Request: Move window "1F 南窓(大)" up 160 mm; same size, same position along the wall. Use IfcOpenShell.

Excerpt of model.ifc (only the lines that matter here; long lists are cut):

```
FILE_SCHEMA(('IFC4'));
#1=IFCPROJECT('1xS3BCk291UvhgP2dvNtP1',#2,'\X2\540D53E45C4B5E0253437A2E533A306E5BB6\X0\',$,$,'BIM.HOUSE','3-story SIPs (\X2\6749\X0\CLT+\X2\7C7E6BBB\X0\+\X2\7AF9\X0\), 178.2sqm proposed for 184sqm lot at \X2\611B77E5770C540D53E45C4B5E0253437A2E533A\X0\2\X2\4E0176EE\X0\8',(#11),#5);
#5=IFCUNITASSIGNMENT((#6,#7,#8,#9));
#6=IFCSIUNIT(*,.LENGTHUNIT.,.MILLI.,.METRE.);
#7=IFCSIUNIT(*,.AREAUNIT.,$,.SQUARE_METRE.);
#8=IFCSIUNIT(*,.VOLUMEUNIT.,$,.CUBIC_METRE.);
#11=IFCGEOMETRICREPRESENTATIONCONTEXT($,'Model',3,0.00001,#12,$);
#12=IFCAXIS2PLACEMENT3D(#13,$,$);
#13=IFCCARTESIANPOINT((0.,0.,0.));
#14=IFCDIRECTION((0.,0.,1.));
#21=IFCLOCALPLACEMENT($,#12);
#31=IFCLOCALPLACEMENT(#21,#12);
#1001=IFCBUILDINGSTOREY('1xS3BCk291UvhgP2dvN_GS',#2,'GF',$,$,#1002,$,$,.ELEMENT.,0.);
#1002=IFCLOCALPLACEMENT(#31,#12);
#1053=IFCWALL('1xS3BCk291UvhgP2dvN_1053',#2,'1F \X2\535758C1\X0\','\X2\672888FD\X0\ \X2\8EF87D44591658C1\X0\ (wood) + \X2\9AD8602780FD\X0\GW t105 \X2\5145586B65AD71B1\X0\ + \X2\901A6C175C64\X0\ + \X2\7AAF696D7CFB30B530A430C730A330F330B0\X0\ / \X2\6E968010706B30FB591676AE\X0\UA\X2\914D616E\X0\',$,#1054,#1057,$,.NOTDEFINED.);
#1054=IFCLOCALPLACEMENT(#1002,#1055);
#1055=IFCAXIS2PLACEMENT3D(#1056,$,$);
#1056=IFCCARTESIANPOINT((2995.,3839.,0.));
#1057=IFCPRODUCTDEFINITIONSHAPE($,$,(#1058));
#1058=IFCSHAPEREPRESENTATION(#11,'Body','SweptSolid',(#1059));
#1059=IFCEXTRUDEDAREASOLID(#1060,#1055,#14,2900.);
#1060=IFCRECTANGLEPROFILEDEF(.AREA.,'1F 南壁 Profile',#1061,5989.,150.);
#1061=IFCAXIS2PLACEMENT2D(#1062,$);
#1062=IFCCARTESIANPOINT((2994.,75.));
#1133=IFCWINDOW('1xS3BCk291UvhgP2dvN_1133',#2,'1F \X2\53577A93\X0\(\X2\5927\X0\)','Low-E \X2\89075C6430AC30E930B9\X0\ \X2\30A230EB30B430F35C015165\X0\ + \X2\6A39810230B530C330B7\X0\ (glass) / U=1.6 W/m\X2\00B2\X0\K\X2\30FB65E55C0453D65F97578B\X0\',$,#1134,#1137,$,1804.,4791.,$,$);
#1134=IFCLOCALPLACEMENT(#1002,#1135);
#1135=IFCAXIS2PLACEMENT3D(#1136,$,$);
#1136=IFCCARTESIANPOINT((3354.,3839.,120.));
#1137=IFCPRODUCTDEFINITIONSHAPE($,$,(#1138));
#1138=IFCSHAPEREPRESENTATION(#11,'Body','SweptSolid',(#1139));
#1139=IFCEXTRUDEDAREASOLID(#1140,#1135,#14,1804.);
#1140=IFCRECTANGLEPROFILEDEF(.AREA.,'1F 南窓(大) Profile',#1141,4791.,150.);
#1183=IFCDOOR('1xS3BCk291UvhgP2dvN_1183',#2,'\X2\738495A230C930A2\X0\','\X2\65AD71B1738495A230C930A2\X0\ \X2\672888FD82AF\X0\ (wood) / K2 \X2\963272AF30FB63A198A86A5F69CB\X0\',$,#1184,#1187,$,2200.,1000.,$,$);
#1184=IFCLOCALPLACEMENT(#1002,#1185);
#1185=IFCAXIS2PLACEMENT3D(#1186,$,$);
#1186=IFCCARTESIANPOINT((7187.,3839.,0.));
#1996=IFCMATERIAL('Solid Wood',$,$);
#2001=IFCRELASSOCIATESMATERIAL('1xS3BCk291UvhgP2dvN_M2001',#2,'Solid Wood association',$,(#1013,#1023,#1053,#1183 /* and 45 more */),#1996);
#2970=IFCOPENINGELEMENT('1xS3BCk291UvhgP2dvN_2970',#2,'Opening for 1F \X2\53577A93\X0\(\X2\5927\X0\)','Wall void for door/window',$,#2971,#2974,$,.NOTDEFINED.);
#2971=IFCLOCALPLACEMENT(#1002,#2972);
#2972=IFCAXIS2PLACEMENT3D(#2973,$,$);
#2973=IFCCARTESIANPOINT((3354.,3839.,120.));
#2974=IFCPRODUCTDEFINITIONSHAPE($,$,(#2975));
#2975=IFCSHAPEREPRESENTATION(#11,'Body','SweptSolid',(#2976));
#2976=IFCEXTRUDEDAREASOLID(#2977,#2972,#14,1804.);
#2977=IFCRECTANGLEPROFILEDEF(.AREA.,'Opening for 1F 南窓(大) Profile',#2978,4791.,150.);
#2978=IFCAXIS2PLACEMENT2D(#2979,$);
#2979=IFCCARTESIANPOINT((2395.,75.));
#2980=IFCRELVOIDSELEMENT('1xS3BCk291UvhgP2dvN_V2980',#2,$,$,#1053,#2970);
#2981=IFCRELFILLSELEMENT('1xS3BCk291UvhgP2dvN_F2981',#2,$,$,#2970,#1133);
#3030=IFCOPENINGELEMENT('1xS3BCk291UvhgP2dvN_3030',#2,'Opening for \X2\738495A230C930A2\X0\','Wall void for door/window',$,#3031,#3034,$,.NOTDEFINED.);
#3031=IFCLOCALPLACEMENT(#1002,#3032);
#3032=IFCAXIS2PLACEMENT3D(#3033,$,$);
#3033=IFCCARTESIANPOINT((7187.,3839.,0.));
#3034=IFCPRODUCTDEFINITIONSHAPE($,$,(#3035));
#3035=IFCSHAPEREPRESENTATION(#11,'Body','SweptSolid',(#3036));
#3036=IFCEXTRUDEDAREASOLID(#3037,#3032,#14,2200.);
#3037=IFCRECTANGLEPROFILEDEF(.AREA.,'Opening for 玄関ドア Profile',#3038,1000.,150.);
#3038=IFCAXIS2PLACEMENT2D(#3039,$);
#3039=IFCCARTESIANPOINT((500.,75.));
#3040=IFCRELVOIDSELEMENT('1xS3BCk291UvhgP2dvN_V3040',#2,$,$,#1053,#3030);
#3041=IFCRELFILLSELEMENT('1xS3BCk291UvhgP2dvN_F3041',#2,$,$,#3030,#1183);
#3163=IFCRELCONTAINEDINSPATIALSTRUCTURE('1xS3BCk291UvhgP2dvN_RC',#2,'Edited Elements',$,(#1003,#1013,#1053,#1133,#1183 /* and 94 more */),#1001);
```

```python
import numpy as np
import ifcopenshell
import ifcopenshell.api.geometry
import ifcopenshell.util.placement
import ifcopenshell.util.unit

model = ifcopenshell.open("model.ifc")
unit_scale = ifcopenshell.util.unit.calculate_unit_scale(model)

window = model.by_guid("1xS3BCk291UvhgP2dvN_1133")
opening = window.FillsVoids[0].RelatingOpeningElement
dz = 0.16 / unit_scale

shift = np.array([0.0, 0.0, dz])
# The window is not placed relative to its opening, so move both.
for product in (opening, window):
    matrix = ifcopenshell.util.placement.get_local_placement(product.ObjectPlacement)
    matrix[:3, 3] += shift
    ifcopenshell.api.geometry.edit_object_placement(model, product=product, matrix=matrix, is_si=False)

print(f"moved by {dz * unit_scale:+.3f} m")

model.write("model_rev.ifc")
```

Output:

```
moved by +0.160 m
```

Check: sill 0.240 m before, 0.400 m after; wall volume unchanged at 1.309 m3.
